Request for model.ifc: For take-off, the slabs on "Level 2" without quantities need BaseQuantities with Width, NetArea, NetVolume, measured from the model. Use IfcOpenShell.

First a look at what the model holds.

```python
import ifcopenshell
import ifcopenshell.util.element
import ifcopenshell.util.unit

model = ifcopenshell.open("model.ifc")
print(model.schema)
for unit_type in ("LENGTHUNIT", "AREAUNIT", "VOLUMEUNIT"):
    print(unit_type, ifcopenshell.util.unit.calculate_unit_scale(model, unit_type))
storey = next(s for s in model.by_type("IfcBuildingStorey") if s.Name == "Level 2")
slabs = [e for e in ifcopenshell.util.element.get_decomposition(storey) if e.is_a("IfcSlab")]
for e in sorted(slabs, key=lambda e: e.id()):
    print(e.id(), e.is_a(), e.Name, list(ifcopenshell.util.element.get_psets(e, qtos_only=True)), sep=" | ")
```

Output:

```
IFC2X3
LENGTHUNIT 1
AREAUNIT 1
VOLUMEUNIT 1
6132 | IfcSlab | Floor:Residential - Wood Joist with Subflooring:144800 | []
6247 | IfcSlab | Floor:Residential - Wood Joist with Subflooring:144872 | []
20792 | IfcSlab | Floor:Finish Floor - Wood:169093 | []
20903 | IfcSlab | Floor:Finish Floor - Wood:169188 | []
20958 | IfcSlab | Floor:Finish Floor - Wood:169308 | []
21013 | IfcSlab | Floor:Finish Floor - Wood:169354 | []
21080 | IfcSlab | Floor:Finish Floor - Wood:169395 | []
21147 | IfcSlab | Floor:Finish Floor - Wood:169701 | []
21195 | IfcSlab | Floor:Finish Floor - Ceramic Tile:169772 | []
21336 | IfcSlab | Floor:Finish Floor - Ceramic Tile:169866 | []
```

```python
import ifcopenshell
import ifcopenshell.api.pset
import ifcopenshell.geom
import ifcopenshell.util.element
import ifcopenshell.util.shape
import ifcopenshell.util.unit

model = ifcopenshell.open("model.ifc")
unit_scale = ifcopenshell.util.unit.calculate_unit_scale(model)
area_scale = ifcopenshell.util.unit.calculate_unit_scale(model, "AREAUNIT")
volume_scale = ifcopenshell.util.unit.calculate_unit_scale(model, "VOLUMEUNIT")
settings = ifcopenshell.geom.settings()

storey = next(s for s in model.by_type("IfcBuildingStorey") if s.Name == "Level 2")
slabs = [e for e in ifcopenshell.util.element.get_decomposition(storey) if e.is_a("IfcSlab")]

for e in sorted(slabs, key=lambda e: e.id()):
    if ifcopenshell.util.element.get_psets(e, qtos_only=True, should_inherit=False):
        continue
    # Geometry comes back in metres, in the element's own axes.
    shape = ifcopenshell.geom.create_shape(settings, e)
    values = {
        "Width": ifcopenshell.util.shape.get_z(shape.geometry) / unit_scale,
        "NetArea": ifcopenshell.util.shape.get_footprint_area(shape.geometry) / area_scale,
        "NetVolume": ifcopenshell.util.shape.get_volume(shape.geometry) / volume_scale,
    }
    qto = ifcopenshell.api.pset.add_qto(model, product=e, name="BaseQuantities")
    ifcopenshell.api.pset.edit_qto(model, qto=qto, properties=values)
    print(e.id(), {k: round(v, 3) for k, v in values.items()})

model.write("model_edited.ifc")
```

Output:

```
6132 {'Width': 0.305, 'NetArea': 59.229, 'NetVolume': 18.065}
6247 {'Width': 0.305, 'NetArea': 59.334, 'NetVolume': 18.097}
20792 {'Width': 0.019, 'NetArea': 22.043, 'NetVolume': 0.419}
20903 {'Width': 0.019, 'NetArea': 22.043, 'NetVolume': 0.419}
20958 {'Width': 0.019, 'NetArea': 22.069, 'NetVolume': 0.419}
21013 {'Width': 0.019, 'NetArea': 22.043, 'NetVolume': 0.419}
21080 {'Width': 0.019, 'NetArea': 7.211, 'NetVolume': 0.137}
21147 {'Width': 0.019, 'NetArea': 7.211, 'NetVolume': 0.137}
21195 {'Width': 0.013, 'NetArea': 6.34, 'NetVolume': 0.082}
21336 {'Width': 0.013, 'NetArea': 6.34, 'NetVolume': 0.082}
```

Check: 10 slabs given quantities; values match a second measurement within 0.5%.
